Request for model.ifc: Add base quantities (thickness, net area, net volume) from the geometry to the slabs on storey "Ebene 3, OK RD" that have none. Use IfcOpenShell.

First a look at what the model holds.

```python
import ifcopenshell
import ifcopenshell.util.element
import ifcopenshell.util.unit

model = ifcopenshell.open("model.ifc")
print(model.schema)
for unit_type in ("LENGTHUNIT", "AREAUNIT", "VOLUMEUNIT"):
    print(unit_type, ifcopenshell.util.unit.calculate_unit_scale(model, unit_type))
storey = next(s for s in model.by_type("IfcBuildingStorey") if s.Name == "Ebene 3, OK RD")
slabs = [e for e in ifcopenshell.util.element.get_decomposition(storey) if e.is_a("IfcSlab")]
for e in sorted(slabs, key=lambda e: e.id()):
    print(e.id(), e.is_a(), e.Name, list(ifcopenshell.util.element.get_psets(e, qtos_only=True)), sep=" | ")
```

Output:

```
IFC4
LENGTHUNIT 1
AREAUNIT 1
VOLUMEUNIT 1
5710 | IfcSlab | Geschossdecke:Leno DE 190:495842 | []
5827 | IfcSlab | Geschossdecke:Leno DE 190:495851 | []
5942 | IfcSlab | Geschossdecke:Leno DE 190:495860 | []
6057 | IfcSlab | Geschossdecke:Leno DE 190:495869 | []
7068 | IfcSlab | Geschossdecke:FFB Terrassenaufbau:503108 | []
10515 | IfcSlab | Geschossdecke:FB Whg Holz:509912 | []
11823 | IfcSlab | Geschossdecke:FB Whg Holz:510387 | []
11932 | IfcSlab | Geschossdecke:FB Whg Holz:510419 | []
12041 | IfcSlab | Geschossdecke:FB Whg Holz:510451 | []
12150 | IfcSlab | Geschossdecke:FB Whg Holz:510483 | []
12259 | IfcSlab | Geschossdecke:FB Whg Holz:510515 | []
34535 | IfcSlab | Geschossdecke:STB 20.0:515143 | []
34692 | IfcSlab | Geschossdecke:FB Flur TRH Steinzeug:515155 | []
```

```python
import ifcopenshell
import ifcopenshell.api.pset
import ifcopenshell.geom
import ifcopenshell.util.element
import ifcopenshell.util.shape
import ifcopenshell.util.unit

model = ifcopenshell.open("model.ifc")
unit_scale = ifcopenshell.util.unit.calculate_unit_scale(model)
area_scale = ifcopenshell.util.unit.calculate_unit_scale(model, "AREAUNIT")
volume_scale = ifcopenshell.util.unit.calculate_unit_scale(model, "VOLUMEUNIT")
settings = ifcopenshell.geom.settings()

storey = next(s for s in model.by_type("IfcBuildingStorey") if s.Name == "Ebene 3, OK RD")
slabs = [e for e in ifcopenshell.util.element.get_decomposition(storey) if e.is_a("IfcSlab")]

for e in sorted(slabs, key=lambda e: e.id()):
    if ifcopenshell.util.element.get_psets(e, qtos_only=True, should_inherit=False):
        continue
    # Geometry comes back in metres, in the element's own axes.
    shape = ifcopenshell.geom.create_shape(settings, e)
    values = {
        "Width": ifcopenshell.util.shape.get_z(shape.geometry) / unit_scale,
        "NetArea": ifcopenshell.util.shape.get_footprint_area(shape.geometry) / area_scale,
        "NetVolume": ifcopenshell.util.shape.get_volume(shape.geometry) / volume_scale,
    }
    qto = ifcopenshell.api.pset.add_qto(model, product=e, name="Qto_SlabBaseQuantities")
    ifcopenshell.api.pset.edit_qto(model, qto=qto, properties=values)
    print(e.id(), {k: round(v, 3) for k, v in values.items()})

model.write("model_updated.ifc")
```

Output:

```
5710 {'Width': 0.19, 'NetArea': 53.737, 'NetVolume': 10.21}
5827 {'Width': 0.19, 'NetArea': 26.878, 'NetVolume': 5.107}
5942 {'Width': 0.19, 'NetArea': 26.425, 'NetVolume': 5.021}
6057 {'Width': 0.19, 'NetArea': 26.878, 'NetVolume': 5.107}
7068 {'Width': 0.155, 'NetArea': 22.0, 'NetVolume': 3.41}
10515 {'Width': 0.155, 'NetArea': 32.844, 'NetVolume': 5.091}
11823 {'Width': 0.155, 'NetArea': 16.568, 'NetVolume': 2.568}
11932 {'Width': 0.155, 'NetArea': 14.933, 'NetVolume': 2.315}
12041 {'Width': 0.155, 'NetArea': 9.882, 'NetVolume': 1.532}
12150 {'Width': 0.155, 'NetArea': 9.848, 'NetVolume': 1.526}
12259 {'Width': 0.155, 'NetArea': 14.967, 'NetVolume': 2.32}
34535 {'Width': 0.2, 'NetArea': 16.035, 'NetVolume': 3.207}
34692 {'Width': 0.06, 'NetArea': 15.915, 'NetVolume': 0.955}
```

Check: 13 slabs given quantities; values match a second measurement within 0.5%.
